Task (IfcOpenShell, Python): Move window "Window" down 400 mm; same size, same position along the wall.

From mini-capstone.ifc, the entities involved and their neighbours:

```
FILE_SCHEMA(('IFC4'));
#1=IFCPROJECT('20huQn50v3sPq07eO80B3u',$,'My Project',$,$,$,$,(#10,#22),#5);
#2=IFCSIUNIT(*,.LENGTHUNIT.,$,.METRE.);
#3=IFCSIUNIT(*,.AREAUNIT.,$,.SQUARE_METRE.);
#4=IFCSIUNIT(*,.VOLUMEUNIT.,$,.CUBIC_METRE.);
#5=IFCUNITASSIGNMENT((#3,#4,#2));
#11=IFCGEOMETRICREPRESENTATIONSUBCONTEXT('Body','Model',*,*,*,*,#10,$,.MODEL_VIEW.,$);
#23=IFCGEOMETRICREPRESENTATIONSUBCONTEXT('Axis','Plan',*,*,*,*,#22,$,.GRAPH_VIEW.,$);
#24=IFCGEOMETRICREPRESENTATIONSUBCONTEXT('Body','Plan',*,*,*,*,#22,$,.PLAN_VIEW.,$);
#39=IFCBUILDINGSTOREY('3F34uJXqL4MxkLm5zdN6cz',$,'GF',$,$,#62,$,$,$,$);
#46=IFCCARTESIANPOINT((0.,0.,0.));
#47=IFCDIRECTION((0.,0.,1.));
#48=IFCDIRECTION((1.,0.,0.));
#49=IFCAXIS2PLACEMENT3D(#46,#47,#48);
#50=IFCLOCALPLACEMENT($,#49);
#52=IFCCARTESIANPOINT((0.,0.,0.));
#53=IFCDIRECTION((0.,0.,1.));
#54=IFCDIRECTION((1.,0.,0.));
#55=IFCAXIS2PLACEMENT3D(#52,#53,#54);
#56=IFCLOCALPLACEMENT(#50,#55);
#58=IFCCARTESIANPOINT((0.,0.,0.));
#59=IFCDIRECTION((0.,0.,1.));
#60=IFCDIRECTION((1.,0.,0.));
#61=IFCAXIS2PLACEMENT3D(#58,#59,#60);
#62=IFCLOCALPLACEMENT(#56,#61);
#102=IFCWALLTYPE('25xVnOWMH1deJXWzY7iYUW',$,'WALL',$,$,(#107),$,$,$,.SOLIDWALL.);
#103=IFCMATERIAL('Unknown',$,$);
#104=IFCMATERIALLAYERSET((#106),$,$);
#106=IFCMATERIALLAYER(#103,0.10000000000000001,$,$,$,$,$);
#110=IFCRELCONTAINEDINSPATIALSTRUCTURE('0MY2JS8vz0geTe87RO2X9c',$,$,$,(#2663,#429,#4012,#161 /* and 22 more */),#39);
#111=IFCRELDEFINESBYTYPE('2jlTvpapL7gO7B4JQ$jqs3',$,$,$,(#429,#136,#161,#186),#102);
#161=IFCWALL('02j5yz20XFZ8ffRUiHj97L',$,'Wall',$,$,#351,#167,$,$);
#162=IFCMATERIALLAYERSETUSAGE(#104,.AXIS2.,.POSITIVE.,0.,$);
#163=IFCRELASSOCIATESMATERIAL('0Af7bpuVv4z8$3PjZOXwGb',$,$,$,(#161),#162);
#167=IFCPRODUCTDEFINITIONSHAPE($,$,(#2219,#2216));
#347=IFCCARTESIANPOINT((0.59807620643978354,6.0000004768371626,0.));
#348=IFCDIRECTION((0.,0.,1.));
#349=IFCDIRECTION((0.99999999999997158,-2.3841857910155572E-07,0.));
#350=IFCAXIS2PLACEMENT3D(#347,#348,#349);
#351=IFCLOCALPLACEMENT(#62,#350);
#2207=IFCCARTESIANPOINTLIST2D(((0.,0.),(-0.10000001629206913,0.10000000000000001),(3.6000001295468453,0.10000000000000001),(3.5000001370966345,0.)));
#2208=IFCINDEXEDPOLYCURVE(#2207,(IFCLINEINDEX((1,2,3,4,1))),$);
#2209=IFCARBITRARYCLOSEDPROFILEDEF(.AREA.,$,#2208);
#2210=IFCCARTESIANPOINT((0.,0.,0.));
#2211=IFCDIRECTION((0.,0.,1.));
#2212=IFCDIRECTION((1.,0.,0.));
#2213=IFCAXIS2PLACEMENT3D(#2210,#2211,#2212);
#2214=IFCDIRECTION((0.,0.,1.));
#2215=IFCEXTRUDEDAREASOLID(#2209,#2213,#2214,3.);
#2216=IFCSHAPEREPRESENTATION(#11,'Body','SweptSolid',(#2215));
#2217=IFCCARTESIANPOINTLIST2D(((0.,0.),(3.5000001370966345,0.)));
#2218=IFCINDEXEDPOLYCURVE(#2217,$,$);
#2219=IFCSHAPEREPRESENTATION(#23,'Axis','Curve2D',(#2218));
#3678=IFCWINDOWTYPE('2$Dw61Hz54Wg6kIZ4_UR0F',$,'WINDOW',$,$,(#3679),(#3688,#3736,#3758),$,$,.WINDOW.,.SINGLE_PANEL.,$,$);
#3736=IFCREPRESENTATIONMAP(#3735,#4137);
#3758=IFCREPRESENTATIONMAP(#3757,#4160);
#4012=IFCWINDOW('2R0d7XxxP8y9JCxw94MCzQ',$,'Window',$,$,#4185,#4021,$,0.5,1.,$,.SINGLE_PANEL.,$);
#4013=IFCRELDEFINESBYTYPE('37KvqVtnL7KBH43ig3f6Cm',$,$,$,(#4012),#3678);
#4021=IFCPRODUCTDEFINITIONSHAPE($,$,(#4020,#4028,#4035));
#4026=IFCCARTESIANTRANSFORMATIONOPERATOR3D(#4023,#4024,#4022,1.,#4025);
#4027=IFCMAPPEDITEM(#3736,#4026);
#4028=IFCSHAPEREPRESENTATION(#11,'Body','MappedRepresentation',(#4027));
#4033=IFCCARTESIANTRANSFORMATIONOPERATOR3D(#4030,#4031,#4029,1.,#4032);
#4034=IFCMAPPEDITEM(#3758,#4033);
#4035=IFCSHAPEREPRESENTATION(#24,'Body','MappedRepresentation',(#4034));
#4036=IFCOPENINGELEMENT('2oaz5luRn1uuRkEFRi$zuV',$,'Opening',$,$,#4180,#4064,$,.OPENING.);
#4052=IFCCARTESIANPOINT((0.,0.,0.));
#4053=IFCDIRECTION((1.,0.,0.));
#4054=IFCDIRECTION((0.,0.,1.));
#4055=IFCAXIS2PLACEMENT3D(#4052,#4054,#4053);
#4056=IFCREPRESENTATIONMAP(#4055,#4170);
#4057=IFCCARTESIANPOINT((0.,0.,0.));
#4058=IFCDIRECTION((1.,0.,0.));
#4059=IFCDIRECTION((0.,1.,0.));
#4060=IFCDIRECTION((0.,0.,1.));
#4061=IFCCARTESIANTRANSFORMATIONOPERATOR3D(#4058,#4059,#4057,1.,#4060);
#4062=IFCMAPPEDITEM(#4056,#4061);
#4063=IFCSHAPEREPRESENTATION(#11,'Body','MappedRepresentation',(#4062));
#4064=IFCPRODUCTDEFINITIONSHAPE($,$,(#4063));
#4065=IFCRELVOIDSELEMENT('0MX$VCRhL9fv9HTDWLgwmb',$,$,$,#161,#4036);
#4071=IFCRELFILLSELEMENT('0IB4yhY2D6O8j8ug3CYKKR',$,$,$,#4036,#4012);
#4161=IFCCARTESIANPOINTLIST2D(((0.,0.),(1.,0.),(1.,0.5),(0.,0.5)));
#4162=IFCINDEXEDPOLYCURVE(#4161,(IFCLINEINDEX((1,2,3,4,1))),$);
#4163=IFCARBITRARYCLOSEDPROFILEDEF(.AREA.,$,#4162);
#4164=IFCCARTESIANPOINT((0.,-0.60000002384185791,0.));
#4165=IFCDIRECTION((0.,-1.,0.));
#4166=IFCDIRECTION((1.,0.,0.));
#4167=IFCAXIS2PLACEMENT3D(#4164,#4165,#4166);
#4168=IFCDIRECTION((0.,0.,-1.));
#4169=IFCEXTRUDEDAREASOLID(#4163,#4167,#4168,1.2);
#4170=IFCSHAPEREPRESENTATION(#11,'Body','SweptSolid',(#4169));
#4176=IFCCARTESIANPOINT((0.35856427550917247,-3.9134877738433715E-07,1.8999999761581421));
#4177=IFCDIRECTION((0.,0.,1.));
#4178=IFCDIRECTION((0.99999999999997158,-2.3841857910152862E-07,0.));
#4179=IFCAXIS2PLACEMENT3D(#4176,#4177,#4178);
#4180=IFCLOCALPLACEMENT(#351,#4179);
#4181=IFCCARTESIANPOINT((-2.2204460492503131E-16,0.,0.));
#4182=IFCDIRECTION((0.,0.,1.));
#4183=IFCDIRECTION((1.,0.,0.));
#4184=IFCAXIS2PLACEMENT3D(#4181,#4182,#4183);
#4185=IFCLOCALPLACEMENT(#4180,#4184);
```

```python
import numpy as np
import ifcopenshell
import ifcopenshell.api.geometry
import ifcopenshell.util.placement
import ifcopenshell.util.unit

model = ifcopenshell.open("mini-capstone.ifc")
unit_scale = ifcopenshell.util.unit.calculate_unit_scale(model)

window = model.by_id(4012)
opening = window.FillsVoids[0].RelatingOpeningElement
dz = -0.4 / unit_scale

shift = np.array([0.0, 0.0, dz])
# The window is placed relative to its opening, so it follows when the opening moves.
matrix = ifcopenshell.util.placement.get_local_placement(opening.ObjectPlacement)
matrix[:3, 3] += shift
ifcopenshell.api.geometry.edit_object_placement(
    model, product=opening, matrix=matrix, is_si=False, should_transform_children=True
)

print(f"moved by {dz * unit_scale:+.3f} m")

model.write("mini-capstone-out.ifc")
```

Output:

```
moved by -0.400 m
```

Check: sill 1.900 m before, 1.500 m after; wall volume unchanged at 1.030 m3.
